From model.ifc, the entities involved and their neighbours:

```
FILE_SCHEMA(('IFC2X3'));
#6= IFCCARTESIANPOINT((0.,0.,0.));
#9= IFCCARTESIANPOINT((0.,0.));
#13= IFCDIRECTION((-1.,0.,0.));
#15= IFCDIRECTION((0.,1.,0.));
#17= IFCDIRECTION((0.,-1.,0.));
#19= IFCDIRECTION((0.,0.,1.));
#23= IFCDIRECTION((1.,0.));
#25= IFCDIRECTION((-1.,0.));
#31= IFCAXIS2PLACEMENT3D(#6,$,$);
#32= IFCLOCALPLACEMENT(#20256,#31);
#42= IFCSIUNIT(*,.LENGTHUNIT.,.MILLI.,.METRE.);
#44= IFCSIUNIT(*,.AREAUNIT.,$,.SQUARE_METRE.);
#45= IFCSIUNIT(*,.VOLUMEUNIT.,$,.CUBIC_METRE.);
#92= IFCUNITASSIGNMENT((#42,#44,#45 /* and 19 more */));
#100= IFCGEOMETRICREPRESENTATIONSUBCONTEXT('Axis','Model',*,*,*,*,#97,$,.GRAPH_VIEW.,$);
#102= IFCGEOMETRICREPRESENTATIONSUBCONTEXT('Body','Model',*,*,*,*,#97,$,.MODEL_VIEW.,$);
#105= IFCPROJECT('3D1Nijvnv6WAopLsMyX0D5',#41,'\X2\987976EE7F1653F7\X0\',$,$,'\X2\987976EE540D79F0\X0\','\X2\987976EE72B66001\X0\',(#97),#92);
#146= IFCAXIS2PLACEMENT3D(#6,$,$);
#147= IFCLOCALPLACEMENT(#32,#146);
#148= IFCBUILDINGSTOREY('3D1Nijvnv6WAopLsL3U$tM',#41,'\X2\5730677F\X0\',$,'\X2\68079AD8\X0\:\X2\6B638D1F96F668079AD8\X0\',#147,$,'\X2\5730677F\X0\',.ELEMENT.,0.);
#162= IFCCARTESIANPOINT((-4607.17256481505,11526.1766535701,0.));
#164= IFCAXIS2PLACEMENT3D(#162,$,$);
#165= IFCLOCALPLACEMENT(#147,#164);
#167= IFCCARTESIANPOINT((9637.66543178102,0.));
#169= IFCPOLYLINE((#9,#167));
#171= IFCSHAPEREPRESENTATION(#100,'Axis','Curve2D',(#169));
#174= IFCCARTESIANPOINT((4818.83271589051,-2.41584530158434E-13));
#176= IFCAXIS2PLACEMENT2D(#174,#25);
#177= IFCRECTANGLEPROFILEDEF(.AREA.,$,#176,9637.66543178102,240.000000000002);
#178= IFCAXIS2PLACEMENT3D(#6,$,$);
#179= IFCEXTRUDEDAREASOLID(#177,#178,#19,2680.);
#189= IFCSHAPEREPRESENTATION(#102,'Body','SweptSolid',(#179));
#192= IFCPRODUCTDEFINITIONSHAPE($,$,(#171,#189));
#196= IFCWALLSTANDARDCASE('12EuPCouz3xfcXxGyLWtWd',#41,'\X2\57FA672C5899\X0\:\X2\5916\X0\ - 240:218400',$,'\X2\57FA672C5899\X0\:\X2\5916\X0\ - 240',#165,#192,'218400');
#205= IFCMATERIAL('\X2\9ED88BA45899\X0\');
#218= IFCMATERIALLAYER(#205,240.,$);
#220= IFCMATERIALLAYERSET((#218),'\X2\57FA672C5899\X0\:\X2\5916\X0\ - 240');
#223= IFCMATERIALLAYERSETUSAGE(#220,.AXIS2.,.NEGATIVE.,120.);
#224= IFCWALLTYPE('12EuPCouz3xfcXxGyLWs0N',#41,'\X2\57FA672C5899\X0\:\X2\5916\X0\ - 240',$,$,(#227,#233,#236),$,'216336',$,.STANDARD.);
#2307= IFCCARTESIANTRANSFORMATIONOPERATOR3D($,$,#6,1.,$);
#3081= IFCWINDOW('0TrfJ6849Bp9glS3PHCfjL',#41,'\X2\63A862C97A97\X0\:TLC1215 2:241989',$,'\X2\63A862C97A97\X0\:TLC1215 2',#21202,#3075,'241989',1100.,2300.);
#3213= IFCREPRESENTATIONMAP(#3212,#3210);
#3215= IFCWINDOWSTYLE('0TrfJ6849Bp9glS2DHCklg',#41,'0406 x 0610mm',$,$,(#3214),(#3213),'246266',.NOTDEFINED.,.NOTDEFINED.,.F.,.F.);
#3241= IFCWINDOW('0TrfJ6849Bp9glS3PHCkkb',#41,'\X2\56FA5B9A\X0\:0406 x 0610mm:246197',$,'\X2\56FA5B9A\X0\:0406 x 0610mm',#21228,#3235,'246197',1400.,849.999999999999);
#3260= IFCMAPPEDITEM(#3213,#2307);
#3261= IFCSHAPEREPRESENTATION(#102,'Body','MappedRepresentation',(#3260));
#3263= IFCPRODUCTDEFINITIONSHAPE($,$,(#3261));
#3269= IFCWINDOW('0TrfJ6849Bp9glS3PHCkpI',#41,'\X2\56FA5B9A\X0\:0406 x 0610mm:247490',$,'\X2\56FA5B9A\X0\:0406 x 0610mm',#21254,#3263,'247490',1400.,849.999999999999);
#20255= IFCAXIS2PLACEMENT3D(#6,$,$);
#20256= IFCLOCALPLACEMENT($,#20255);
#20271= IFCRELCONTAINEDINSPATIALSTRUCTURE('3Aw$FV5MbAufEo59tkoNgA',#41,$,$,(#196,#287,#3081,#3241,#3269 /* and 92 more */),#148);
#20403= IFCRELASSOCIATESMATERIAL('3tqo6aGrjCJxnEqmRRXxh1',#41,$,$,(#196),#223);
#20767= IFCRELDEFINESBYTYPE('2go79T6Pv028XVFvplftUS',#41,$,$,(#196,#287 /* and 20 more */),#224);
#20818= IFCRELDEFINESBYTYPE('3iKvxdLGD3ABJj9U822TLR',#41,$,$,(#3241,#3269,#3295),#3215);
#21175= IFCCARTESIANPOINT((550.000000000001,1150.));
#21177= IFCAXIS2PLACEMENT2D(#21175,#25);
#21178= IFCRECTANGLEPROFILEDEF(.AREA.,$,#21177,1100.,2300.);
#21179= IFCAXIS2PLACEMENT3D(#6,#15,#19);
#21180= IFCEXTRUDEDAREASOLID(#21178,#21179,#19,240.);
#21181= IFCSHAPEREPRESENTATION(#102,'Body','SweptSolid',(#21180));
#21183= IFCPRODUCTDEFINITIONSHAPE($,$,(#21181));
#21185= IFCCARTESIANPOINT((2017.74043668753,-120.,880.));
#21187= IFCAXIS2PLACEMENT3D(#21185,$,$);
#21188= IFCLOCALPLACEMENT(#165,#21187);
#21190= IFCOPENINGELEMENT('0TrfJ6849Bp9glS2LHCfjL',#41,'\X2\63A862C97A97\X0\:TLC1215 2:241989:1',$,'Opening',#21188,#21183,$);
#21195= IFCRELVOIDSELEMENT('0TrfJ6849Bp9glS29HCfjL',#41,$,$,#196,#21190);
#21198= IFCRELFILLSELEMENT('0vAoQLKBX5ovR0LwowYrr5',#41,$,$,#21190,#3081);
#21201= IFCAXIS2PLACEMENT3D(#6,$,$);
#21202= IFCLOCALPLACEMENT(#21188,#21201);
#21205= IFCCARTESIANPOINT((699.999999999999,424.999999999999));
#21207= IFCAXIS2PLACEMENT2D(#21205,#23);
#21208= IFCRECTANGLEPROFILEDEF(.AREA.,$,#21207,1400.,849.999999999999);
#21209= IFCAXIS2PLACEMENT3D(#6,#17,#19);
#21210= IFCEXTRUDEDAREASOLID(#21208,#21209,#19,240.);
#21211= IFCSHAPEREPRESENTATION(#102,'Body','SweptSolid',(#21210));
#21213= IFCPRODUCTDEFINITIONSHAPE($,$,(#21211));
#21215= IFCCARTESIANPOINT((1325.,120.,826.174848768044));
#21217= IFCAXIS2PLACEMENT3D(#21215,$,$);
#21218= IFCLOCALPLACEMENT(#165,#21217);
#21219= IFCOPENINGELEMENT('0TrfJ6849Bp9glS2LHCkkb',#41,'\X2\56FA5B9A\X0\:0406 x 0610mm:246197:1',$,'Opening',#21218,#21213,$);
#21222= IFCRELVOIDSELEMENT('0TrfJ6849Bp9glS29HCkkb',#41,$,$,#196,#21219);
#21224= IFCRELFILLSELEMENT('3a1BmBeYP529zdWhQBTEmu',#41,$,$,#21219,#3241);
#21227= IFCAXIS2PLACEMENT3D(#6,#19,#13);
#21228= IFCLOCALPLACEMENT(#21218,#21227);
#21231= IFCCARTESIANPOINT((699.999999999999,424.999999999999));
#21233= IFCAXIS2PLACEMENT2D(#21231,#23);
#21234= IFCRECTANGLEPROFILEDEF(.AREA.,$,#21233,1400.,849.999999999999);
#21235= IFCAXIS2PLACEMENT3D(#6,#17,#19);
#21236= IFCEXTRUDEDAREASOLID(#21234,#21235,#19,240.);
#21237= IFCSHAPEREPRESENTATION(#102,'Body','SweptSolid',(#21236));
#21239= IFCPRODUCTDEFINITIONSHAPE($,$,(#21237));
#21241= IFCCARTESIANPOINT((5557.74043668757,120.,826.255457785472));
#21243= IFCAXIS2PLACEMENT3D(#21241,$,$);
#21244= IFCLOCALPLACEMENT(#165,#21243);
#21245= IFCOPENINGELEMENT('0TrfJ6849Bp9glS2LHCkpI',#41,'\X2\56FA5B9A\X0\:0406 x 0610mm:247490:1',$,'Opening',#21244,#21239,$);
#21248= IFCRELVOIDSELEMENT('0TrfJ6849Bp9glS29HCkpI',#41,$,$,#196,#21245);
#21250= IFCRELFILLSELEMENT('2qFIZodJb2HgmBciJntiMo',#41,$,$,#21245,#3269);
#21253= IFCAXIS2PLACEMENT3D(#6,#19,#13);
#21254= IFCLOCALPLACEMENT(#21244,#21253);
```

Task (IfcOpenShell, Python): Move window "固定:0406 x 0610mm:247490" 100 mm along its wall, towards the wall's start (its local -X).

```python
import ifcopenshell
import ifcopenshell.api.geometry
import ifcopenshell.util.placement
import ifcopenshell.util.unit

model = ifcopenshell.open("model.ifc")
unit_scale = ifcopenshell.util.unit.calculate_unit_scale(model)

window = model.by_guid("0TrfJ6849Bp9glS3PHCkpI")
opening = window.FillsVoids[0].RelatingOpeningElement
wall = opening.VoidsElements[0].RelatingBuildingElement

wall_matrix = ifcopenshell.util.placement.get_local_placement(wall.ObjectPlacement)
shift = wall_matrix[:3, 0] * -0.1 / unit_scale
before = ifcopenshell.util.placement.get_local_placement(window.ObjectPlacement)[:3, 3].copy()

# The window is placed relative to its opening, so it follows when the opening moves.
matrix = ifcopenshell.util.placement.get_local_placement(opening.ObjectPlacement)
matrix[:3, 3] += shift
ifcopenshell.api.geometry.edit_object_placement(
    model, product=opening, matrix=matrix, is_si=False, should_transform_children=True
)

after = ifcopenshell.util.placement.get_local_placement(window.ObjectPlacement)[:3, 3]
print("window moved by", (after - before).round(3) + 0.0)

model.write("model_v2.ifc")
```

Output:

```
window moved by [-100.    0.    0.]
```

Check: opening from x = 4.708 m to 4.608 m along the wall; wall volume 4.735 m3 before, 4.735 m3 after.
